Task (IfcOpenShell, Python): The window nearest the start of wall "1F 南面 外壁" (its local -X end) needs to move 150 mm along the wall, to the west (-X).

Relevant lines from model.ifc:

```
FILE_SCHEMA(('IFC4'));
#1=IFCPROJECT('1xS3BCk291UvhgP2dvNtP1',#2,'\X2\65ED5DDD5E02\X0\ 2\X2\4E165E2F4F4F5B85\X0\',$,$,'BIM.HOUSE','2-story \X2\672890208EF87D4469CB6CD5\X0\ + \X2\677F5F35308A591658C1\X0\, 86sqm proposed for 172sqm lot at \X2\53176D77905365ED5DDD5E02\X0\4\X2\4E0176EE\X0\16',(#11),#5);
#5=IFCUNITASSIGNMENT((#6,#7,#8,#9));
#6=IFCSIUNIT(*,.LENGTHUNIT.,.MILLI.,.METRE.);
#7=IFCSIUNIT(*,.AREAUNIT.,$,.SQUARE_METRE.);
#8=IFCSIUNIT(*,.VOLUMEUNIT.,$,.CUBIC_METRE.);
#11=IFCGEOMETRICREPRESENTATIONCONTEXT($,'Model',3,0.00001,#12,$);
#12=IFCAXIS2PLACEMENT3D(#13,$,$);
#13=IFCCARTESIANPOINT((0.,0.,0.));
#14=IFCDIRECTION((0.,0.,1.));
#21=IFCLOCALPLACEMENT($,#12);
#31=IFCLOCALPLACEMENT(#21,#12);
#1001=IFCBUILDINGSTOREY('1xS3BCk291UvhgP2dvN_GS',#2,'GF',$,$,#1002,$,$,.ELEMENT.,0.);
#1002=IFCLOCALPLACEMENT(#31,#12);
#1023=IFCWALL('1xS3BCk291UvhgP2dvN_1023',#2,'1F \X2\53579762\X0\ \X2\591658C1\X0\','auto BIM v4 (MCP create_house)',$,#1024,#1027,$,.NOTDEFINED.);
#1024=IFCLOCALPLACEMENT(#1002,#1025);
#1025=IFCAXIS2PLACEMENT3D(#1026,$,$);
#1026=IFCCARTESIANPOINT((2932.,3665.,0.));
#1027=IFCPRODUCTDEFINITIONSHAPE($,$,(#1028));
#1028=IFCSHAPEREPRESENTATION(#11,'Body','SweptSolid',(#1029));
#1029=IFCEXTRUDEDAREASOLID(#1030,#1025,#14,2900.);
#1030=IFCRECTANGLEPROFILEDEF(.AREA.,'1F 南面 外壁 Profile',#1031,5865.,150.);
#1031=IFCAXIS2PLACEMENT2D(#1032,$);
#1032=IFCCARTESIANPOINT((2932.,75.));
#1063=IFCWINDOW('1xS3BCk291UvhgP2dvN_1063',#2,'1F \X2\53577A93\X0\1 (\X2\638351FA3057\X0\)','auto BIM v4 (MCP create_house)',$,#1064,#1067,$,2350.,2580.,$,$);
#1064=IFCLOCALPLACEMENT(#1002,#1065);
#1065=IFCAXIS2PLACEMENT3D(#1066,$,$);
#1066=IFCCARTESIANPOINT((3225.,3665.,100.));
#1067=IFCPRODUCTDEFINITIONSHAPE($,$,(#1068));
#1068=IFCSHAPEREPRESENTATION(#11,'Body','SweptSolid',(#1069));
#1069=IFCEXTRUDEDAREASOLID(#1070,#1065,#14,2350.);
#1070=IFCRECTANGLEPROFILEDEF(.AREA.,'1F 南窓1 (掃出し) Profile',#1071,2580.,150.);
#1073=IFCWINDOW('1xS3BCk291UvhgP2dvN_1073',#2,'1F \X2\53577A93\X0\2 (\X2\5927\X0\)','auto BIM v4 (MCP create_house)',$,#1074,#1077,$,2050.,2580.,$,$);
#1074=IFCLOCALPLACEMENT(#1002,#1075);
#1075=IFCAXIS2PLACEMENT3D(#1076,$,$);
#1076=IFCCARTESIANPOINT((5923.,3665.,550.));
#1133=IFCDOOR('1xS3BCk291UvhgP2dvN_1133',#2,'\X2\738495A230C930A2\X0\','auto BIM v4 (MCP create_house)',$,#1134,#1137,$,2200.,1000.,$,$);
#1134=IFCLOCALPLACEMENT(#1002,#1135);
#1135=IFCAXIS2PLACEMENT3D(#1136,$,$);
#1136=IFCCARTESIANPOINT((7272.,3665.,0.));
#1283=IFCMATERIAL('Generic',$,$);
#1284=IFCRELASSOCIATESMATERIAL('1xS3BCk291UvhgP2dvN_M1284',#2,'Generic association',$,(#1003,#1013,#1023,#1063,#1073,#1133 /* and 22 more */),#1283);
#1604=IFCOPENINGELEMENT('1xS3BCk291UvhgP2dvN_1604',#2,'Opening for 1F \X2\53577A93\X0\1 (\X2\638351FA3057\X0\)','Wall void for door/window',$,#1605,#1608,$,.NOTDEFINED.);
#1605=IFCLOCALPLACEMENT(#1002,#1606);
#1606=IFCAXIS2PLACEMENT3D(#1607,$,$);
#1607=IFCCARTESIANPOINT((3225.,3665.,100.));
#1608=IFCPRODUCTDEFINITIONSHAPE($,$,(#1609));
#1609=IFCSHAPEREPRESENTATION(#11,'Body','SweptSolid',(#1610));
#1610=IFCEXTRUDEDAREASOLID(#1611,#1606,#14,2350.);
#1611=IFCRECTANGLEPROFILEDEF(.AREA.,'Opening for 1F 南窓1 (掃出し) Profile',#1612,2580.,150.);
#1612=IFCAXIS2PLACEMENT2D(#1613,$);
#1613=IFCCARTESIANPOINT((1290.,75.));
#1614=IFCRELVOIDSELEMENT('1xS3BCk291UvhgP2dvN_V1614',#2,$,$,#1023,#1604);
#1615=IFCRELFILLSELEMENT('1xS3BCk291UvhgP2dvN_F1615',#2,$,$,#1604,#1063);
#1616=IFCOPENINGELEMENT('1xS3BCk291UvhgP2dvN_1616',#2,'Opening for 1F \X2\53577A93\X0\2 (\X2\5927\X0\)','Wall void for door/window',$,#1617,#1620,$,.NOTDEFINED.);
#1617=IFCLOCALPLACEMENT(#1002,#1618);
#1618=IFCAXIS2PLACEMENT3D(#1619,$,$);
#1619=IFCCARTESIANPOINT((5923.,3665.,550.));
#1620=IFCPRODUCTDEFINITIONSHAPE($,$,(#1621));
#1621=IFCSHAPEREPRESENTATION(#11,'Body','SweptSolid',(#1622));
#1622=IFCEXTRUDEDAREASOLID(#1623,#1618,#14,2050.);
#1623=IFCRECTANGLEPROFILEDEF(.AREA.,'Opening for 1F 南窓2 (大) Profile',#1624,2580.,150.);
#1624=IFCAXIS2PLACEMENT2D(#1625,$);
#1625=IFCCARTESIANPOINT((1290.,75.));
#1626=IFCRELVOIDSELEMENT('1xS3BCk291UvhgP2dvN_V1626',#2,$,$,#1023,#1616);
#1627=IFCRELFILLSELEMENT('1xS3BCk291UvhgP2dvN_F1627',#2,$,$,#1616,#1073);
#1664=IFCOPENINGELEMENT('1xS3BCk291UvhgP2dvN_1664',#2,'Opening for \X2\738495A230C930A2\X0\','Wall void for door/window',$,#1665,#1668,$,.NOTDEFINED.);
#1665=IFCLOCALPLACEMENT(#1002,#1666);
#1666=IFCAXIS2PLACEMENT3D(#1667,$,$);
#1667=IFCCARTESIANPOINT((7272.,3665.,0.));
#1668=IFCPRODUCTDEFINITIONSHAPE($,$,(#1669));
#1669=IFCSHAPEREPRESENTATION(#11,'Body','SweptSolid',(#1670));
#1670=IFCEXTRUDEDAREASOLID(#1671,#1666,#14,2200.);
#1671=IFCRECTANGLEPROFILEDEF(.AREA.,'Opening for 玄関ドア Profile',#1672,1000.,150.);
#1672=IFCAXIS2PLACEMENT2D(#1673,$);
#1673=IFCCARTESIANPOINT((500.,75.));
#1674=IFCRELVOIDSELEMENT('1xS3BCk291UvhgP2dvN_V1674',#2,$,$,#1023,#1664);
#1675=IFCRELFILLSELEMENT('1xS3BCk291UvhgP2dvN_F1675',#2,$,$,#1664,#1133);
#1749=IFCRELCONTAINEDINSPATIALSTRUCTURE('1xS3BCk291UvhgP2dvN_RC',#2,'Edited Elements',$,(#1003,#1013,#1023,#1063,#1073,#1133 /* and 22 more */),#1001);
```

```python
import ifcopenshell
import ifcopenshell.api.geometry
import ifcopenshell.util.placement
import ifcopenshell.util.unit

model = ifcopenshell.open("model.ifc")
unit_scale = ifcopenshell.util.unit.calculate_unit_scale(model)

window = model.by_id(1063)
opening = window.FillsVoids[0].RelatingOpeningElement
wall = opening.VoidsElements[0].RelatingBuildingElement

wall_matrix = ifcopenshell.util.placement.get_local_placement(wall.ObjectPlacement)
shift = wall_matrix[:3, 0] * -0.15 / unit_scale
before = ifcopenshell.util.placement.get_local_placement(window.ObjectPlacement)[:3, 3].copy()

# The window is not placed relative to its opening, so move both.
for product in (opening, window):
    matrix = ifcopenshell.util.placement.get_local_placement(product.ObjectPlacement)
    matrix[:3, 3] += shift
    ifcopenshell.api.geometry.edit_object_placement(model, product=product, matrix=matrix, is_si=False)

after = ifcopenshell.util.placement.get_local_placement(window.ObjectPlacement)[:3, 3]
print("window moved by", (after - before).round(3) + 0.0)

model.write("model_rev.ifc")
```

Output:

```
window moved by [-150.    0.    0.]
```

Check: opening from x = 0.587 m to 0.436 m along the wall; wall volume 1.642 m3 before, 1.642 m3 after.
